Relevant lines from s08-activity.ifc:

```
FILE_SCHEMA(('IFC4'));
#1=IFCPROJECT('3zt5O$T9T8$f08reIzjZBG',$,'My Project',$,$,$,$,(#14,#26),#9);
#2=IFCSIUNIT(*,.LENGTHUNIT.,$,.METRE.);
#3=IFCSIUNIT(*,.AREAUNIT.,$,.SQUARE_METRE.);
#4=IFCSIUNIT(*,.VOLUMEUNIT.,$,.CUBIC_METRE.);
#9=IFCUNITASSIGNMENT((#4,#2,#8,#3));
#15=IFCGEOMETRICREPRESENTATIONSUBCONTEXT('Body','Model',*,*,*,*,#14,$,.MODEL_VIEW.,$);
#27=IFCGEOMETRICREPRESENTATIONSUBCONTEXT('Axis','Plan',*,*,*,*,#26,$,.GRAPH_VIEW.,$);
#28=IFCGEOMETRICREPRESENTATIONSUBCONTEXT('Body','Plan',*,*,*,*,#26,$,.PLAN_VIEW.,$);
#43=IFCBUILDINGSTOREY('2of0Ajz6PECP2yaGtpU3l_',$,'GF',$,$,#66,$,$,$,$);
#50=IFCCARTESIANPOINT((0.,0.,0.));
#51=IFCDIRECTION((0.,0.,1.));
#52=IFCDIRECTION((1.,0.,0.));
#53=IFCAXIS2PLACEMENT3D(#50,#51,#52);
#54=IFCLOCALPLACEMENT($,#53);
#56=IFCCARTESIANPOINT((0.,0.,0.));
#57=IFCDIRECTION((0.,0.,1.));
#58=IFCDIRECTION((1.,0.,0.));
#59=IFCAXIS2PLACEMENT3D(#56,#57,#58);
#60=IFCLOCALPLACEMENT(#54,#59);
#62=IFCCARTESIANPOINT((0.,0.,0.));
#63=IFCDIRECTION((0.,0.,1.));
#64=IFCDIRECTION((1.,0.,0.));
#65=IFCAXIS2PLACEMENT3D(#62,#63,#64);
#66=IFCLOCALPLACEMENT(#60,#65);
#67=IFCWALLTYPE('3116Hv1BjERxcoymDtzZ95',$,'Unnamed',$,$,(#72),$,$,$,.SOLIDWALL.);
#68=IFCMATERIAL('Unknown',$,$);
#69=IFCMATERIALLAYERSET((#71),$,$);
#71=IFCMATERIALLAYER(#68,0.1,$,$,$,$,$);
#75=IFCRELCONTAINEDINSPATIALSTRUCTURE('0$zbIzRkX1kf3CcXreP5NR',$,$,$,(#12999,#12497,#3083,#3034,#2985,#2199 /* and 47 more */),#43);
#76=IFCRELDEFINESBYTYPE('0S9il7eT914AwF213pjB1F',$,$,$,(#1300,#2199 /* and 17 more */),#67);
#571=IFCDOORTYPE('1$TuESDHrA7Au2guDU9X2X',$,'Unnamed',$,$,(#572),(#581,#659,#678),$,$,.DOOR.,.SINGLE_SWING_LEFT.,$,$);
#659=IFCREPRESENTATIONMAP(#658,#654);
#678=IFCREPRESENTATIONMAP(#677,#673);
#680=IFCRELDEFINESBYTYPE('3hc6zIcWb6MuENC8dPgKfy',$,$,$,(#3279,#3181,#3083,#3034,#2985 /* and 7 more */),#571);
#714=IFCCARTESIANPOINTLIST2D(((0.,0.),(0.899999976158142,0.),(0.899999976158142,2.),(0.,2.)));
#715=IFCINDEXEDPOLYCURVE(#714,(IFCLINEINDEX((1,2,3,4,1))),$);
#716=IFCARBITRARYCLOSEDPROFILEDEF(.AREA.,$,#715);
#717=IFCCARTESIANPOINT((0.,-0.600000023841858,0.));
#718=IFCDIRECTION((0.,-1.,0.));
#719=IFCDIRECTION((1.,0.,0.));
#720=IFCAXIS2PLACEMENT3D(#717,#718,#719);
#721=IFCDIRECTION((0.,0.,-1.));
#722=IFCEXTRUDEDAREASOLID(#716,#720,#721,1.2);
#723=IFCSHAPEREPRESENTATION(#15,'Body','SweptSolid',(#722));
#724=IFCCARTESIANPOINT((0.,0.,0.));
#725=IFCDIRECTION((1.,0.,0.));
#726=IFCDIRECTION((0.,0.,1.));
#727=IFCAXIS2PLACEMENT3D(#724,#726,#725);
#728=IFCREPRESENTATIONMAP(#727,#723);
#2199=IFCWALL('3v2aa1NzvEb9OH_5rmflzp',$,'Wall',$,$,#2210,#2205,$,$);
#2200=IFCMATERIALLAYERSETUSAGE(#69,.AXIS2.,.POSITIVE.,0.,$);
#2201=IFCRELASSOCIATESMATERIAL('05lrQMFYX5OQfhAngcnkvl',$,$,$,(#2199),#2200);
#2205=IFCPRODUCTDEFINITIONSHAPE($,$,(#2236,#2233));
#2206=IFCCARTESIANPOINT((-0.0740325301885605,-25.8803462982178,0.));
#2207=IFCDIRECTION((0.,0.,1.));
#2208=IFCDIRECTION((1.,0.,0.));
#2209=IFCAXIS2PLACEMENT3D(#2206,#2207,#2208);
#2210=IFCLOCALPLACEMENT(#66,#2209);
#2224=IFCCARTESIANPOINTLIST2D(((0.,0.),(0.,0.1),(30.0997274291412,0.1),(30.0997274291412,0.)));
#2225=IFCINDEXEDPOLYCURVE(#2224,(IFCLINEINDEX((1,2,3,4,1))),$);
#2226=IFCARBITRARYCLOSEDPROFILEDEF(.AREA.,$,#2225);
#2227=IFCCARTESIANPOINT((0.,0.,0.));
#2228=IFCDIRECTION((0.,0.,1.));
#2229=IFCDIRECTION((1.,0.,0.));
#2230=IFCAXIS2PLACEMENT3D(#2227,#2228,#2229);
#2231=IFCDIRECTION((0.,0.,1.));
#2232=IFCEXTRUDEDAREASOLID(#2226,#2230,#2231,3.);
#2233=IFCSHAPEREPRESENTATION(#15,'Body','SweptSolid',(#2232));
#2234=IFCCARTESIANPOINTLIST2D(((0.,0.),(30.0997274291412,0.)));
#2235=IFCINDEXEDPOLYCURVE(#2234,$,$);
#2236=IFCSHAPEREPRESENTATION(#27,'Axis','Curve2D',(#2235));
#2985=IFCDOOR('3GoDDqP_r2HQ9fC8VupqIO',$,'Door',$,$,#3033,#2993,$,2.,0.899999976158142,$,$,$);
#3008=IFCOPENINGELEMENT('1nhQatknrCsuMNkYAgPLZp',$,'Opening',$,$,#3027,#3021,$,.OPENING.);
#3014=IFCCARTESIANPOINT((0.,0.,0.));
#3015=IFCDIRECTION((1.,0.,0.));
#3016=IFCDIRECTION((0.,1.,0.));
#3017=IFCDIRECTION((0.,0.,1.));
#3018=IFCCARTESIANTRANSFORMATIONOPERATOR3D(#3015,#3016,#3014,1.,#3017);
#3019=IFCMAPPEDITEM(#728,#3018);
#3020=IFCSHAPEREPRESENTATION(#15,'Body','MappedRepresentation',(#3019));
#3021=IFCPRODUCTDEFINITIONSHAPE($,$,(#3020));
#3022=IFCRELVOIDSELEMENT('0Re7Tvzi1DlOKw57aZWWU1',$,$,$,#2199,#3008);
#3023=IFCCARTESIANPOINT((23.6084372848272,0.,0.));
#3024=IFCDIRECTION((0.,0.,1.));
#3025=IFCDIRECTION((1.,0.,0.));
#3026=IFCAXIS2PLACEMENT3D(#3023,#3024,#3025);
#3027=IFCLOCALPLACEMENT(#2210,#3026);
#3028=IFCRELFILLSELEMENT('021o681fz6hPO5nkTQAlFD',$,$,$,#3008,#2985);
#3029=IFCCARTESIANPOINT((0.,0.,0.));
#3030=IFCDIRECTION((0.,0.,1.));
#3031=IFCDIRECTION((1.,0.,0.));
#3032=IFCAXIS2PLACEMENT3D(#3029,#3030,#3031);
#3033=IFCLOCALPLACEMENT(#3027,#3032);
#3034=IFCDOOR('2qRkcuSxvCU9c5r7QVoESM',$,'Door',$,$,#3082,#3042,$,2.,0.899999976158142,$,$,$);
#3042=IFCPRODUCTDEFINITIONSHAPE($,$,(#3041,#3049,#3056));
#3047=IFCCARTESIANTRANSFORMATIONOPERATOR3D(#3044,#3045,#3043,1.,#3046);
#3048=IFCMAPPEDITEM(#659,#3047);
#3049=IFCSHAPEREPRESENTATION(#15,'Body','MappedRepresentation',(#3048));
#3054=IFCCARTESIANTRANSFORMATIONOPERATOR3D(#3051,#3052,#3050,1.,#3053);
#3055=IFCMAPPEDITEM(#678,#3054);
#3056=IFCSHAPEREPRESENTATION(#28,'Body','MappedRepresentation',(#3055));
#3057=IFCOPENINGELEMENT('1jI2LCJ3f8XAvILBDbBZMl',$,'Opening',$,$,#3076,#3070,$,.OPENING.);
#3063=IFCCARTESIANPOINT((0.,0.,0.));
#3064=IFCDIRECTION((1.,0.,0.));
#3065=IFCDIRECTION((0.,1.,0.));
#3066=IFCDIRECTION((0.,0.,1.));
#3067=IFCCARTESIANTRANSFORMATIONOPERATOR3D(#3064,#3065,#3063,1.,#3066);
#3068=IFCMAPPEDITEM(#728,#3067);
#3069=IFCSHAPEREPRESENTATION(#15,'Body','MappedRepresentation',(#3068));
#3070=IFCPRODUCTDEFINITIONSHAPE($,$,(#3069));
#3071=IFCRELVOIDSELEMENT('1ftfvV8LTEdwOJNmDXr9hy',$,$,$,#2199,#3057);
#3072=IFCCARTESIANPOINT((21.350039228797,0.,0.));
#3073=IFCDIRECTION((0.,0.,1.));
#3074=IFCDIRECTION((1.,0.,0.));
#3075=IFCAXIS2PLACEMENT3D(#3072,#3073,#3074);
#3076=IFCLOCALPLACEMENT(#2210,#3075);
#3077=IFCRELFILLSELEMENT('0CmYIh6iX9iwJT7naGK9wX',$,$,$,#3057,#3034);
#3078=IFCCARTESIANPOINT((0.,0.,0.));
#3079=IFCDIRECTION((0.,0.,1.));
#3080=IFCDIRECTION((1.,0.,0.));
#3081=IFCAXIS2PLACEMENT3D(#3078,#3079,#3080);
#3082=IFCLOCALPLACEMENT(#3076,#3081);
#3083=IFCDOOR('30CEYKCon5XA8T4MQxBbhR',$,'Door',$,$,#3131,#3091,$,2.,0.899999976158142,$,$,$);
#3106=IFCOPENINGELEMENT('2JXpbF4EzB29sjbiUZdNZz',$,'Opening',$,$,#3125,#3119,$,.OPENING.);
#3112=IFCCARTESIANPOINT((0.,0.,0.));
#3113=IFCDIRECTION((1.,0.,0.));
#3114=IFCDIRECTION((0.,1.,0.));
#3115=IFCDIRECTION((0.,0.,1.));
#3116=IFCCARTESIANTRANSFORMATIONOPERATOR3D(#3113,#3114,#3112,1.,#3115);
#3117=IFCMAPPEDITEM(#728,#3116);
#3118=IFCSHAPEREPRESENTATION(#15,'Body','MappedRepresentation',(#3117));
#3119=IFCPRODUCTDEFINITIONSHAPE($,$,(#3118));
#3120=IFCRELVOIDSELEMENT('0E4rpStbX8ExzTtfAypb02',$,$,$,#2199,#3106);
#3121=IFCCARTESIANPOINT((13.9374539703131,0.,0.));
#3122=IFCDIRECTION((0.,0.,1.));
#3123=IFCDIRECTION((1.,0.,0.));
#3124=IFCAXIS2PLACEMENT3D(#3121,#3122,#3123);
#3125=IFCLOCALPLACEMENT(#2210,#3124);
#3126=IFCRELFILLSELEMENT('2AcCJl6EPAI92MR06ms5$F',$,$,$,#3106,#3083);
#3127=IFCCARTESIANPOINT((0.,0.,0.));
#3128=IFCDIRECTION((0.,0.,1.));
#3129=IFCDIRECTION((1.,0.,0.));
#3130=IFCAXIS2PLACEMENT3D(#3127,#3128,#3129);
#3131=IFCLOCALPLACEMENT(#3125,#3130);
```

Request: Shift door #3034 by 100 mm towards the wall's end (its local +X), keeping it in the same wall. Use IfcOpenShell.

```python
import ifcopenshell
import ifcopenshell.api.geometry
import ifcopenshell.util.placement
import ifcopenshell.util.unit

model = ifcopenshell.open("s08-activity.ifc")
unit_scale = ifcopenshell.util.unit.calculate_unit_scale(model)

door = model.by_guid("2qRkcuSxvCU9c5r7QVoESM")
opening = door.FillsVoids[0].RelatingOpeningElement
wall = opening.VoidsElements[0].RelatingBuildingElement

wall_matrix = ifcopenshell.util.placement.get_local_placement(wall.ObjectPlacement)
shift = wall_matrix[:3, 0] * 0.1 / unit_scale
before = ifcopenshell.util.placement.get_local_placement(door.ObjectPlacement)[:3, 3].copy()

# The door is placed relative to its opening, so it follows when the opening moves.
matrix = ifcopenshell.util.placement.get_local_placement(opening.ObjectPlacement)
matrix[:3, 3] += shift
ifcopenshell.api.geometry.edit_object_placement(
    model, product=opening, matrix=matrix, is_si=False, should_transform_children=True
)

after = ifcopenshell.util.placement.get_local_placement(door.ObjectPlacement)[:3, 3]
print("door moved by", (after - before).round(3) + 0.0)

model.write("s08-activity_rev.ifc")
```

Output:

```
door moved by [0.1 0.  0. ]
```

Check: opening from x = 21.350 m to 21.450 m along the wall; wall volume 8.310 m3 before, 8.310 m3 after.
